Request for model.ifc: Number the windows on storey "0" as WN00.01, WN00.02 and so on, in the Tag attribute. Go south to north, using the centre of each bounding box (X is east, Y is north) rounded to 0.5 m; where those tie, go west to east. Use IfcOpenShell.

First a look at what the model holds.

```python
import ifcopenshell
import ifcopenshell.util.element
import ifcopenshell.util.placement

model = ifcopenshell.open("model.ifc")
print(model.schema)
storey = next(s for s in model.by_type("IfcBuildingStorey") if s.Name == "0")
windows = [e for e in ifcopenshell.util.element.get_decomposition(storey) if e.is_a("IfcWindow")]
for e in sorted(windows, key=lambda e: e.id()):
    origin = ifcopenshell.util.placement.get_local_placement(e.ObjectPlacement)[:3, 3]
    print(e.id(), e.Tag, e.Name, origin.round(2) + 0.0, sep=" | ")
```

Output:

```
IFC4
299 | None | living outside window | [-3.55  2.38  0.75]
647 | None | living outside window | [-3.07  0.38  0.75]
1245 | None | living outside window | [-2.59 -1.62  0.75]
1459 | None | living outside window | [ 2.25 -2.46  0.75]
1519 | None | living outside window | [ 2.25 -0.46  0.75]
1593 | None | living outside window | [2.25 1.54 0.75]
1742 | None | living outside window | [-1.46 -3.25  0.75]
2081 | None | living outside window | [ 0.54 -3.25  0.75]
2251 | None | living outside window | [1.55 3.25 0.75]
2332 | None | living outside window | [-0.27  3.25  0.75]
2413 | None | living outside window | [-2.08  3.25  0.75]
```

```python
import ifcopenshell
import ifcopenshell.geom
import ifcopenshell.util.element
import ifcopenshell.util.shape

model = ifcopenshell.open("model.ifc")
settings = ifcopenshell.geom.settings()
settings.set("use-world-coords", True)


def centre(element):
    shape = ifcopenshell.geom.create_shape(settings, element)
    return ifcopenshell.util.shape.get_bbox_centroid(shape.geometry)


storey = next(s for s in model.by_type("IfcBuildingStorey") if s.Name == "0")
windows = [e for e in ifcopenshell.util.element.get_decomposition(storey) if e.is_a("IfcWindow")]

# Insertion points can sit at a corner or the storey origin, so sort by the geometry (in metres).
centres = {e: centre(e) for e in windows}
windows.sort(key=lambda e: (round(centres[e][1] / 0.5), centres[e][0]))

for i, e in enumerate(windows, start=1):
    number = f"WN00.{i:02d}"
    e.Tag = number
    print(e.id(), number)

model.write("model_edited.ifc")
```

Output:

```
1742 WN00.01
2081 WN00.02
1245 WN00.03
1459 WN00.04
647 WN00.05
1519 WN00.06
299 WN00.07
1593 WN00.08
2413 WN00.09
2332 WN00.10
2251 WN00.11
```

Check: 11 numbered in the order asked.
